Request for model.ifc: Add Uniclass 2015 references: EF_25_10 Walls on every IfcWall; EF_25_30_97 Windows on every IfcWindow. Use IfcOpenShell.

First a look at what the model holds.

```python
import ifcopenshell

model = ifcopenshell.open("model.ifc")
print(model.schema)
print("classifications:", [c.Name for c in model.by_type("IfcClassification")])
for ifc_class in ("IfcDoor", "IfcRoof", "IfcStair", "IfcWall", "IfcWindow"):
    print(ifc_class, len(model.by_type(ifc_class)))
```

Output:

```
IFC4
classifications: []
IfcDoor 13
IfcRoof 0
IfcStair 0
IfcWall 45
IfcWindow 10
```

```python
import ifcopenshell
import ifcopenshell.api.classification

model = ifcopenshell.open("model.ifc")

system = ifcopenshell.api.classification.add_classification(model, classification="Uniclass 2015")

codes = {
    "IfcWall": ("EF_25_10", "Walls"),
    "IfcWindow": ("EF_25_30_97", "Windows"),
}
for ifc_class, (code, name) in codes.items():
    products = model.by_type(ifc_class)
    ifcopenshell.api.classification.add_reference(
        model, products=products, classification=system, identification=code, name=name
    )
    print(code, len(products))

model.write("model_edited.ifc")
```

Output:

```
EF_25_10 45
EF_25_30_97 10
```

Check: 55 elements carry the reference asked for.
